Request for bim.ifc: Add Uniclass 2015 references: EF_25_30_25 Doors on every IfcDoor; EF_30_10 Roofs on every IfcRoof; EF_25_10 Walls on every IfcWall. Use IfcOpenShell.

First a look at what the model holds.

```python
import ifcopenshell

model = ifcopenshell.open("bim.ifc")
print(model.schema)
print("classifications:", [c.Name for c in model.by_type("IfcClassification")])
for ifc_class in ("IfcDoor", "IfcRoof", "IfcStair", "IfcWall", "IfcWindow"):
    print(ifc_class, len(model.by_type(ifc_class)))
```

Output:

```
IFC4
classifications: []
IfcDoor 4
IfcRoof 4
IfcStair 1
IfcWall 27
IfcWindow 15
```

```python
import ifcopenshell
import ifcopenshell.api.classification

model = ifcopenshell.open("bim.ifc")

system = ifcopenshell.api.classification.add_classification(model, classification="Uniclass 2015")

codes = {
    "IfcDoor": ("EF_25_30_25", "Doors"),
    "IfcRoof": ("EF_30_10", "Roofs"),
    "IfcWall": ("EF_25_10", "Walls"),
}
for ifc_class, (code, name) in codes.items():
    products = model.by_type(ifc_class)
    ifcopenshell.api.classification.add_reference(
        model, products=products, classification=system, identification=code, name=name
    )
    print(code, len(products))

model.write("bim_updated.ifc")
```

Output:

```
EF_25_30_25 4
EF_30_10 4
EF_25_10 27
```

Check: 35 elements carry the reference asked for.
